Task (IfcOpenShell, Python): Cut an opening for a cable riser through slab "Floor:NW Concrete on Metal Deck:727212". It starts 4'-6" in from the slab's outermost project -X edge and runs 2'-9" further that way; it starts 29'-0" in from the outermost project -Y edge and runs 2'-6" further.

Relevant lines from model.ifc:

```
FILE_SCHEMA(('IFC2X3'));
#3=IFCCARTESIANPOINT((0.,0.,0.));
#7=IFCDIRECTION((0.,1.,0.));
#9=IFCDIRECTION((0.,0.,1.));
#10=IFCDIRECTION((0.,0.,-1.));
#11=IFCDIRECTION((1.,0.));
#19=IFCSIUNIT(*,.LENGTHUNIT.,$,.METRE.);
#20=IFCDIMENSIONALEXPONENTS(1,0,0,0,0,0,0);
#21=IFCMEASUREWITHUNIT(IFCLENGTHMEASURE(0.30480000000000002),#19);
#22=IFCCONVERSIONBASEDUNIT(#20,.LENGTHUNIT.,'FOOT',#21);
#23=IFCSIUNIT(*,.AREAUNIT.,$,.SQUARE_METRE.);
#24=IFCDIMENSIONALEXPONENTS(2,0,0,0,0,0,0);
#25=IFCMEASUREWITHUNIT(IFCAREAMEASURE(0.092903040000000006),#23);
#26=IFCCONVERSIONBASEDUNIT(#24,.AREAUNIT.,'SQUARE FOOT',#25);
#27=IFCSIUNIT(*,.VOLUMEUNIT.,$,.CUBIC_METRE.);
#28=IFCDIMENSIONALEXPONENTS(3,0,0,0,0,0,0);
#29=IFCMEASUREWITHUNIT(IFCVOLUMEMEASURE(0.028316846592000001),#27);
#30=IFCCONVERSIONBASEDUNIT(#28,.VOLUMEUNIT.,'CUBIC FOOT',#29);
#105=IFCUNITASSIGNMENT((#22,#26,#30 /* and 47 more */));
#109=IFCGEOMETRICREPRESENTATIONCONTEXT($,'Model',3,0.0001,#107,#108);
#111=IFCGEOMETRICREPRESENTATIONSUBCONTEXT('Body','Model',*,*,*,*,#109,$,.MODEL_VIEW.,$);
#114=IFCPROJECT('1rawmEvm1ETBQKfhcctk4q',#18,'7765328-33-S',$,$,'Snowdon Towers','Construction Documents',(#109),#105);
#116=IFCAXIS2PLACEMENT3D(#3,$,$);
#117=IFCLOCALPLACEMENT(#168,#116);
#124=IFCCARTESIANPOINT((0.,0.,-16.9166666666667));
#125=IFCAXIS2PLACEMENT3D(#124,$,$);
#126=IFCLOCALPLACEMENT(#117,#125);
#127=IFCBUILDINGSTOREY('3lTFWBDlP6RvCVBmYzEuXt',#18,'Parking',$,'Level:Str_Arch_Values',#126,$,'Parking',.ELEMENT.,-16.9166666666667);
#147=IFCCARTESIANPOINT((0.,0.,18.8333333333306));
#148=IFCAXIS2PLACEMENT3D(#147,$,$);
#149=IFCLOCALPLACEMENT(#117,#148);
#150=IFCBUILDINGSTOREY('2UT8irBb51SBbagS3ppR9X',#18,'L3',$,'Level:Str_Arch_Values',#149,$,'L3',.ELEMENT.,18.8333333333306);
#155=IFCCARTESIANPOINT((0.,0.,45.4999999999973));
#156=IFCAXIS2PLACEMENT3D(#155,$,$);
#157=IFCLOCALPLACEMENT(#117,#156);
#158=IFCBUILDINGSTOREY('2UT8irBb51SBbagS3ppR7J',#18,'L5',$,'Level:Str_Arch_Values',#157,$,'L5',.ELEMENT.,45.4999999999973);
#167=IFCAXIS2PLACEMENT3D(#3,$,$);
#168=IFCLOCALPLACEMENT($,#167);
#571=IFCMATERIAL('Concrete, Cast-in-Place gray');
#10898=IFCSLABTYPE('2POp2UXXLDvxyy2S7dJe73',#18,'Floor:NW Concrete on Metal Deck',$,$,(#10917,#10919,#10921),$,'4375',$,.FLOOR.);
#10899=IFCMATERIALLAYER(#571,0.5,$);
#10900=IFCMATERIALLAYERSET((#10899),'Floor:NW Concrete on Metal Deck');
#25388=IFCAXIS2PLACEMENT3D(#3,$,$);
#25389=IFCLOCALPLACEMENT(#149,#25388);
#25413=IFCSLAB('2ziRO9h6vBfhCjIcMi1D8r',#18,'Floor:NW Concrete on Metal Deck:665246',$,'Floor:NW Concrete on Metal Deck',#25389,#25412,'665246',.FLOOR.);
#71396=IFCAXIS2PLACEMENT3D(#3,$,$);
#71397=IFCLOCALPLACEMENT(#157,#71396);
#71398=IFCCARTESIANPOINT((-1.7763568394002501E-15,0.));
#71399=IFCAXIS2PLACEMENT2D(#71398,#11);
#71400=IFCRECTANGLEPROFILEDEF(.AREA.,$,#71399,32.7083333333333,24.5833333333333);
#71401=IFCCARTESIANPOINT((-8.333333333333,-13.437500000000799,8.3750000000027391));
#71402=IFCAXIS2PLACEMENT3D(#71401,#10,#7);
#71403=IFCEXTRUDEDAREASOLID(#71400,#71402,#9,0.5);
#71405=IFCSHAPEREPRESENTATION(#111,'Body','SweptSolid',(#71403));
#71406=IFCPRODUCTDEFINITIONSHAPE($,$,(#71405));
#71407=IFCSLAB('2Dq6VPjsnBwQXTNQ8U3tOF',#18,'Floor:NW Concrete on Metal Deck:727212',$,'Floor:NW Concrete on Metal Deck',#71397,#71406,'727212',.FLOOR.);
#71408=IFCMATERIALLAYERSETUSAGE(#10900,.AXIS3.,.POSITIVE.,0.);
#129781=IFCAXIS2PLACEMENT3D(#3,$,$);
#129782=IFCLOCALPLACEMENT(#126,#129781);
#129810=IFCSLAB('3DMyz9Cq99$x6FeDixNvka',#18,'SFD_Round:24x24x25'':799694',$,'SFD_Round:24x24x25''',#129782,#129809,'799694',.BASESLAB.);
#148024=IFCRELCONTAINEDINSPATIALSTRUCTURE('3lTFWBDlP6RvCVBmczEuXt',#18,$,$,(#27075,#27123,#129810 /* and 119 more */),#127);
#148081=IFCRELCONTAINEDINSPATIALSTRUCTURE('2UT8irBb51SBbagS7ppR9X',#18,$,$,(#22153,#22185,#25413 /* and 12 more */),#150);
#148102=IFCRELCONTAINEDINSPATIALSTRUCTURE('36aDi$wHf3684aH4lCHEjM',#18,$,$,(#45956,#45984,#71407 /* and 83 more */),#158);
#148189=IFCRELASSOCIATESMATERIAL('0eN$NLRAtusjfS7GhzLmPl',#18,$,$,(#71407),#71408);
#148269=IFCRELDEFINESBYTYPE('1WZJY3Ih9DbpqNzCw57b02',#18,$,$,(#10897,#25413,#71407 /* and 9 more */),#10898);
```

```python
import numpy as np
import ifcopenshell
import ifcopenshell.api.feature
import ifcopenshell.api.geometry
import ifcopenshell.api.root
import ifcopenshell.geom
import ifcopenshell.util.placement
import ifcopenshell.util.representation
import ifcopenshell.util.shape
import ifcopenshell.util.unit

model = ifcopenshell.open("model.ifc")
unit_scale = ifcopenshell.util.unit.calculate_unit_scale(model)
settings = ifcopenshell.geom.settings()


def volume(element):
    """Net volume in cubic metres, openings subtracted."""
    shape = ifcopenshell.geom.create_shape(settings, element)
    return ifcopenshell.util.shape.get_volume(shape.geometry)


slab = model.by_guid("2Dq6VPjsnBwQXTNQ8U3tOF")
before = volume(slab)

# Extent in the slab's own axes, in metres. The edges named are its -X and -Y sides.
slab_shape = ifcopenshell.geom.create_shape(settings, slab)
vertices = ifcopenshell.util.shape.get_vertices(slab_shape.geometry)
x_min, y_min, bottom = vertices.min(axis=0)
top = vertices[:, 2].max()

opening = ifcopenshell.api.root.create_entity(model, ifc_class="IfcOpeningElement", name="Cable riser opening")
context = ifcopenshell.util.representation.get_context(model, "Model", "Body", "MODEL_VIEW")
width, depth = 0.8382, 0.762
outline = [(0.0, 0.0), (width, 0.0), (width, depth), (0.0, depth), (0.0, 0.0)]
# Overshoot both faces by 50 mm so the cut is clean.
shape = ifcopenshell.api.geometry.add_slab_representation(
    model, context=context, depth=top - bottom + 0.1, polyline=outline
)
ifcopenshell.api.geometry.assign_representation(model, product=opening, representation=shape)

matrix = ifcopenshell.util.placement.get_local_placement(slab.ObjectPlacement)
matrix[:, 3] = matrix @ np.append(np.array([x_min + 1.3716, y_min + 8.8392, bottom - 0.05]) / unit_scale, 1.0)
ifcopenshell.api.geometry.edit_object_placement(model, product=opening, matrix=matrix, is_si=False)
ifcopenshell.api.feature.add_feature(model, feature=opening, element=slab)

after = volume(slab)

print(f"slab volume {before:.3f} -> {after:.3f} m3")

model.write("model_updated.ifc")
```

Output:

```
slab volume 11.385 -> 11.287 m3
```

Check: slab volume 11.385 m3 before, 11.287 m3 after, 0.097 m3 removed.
